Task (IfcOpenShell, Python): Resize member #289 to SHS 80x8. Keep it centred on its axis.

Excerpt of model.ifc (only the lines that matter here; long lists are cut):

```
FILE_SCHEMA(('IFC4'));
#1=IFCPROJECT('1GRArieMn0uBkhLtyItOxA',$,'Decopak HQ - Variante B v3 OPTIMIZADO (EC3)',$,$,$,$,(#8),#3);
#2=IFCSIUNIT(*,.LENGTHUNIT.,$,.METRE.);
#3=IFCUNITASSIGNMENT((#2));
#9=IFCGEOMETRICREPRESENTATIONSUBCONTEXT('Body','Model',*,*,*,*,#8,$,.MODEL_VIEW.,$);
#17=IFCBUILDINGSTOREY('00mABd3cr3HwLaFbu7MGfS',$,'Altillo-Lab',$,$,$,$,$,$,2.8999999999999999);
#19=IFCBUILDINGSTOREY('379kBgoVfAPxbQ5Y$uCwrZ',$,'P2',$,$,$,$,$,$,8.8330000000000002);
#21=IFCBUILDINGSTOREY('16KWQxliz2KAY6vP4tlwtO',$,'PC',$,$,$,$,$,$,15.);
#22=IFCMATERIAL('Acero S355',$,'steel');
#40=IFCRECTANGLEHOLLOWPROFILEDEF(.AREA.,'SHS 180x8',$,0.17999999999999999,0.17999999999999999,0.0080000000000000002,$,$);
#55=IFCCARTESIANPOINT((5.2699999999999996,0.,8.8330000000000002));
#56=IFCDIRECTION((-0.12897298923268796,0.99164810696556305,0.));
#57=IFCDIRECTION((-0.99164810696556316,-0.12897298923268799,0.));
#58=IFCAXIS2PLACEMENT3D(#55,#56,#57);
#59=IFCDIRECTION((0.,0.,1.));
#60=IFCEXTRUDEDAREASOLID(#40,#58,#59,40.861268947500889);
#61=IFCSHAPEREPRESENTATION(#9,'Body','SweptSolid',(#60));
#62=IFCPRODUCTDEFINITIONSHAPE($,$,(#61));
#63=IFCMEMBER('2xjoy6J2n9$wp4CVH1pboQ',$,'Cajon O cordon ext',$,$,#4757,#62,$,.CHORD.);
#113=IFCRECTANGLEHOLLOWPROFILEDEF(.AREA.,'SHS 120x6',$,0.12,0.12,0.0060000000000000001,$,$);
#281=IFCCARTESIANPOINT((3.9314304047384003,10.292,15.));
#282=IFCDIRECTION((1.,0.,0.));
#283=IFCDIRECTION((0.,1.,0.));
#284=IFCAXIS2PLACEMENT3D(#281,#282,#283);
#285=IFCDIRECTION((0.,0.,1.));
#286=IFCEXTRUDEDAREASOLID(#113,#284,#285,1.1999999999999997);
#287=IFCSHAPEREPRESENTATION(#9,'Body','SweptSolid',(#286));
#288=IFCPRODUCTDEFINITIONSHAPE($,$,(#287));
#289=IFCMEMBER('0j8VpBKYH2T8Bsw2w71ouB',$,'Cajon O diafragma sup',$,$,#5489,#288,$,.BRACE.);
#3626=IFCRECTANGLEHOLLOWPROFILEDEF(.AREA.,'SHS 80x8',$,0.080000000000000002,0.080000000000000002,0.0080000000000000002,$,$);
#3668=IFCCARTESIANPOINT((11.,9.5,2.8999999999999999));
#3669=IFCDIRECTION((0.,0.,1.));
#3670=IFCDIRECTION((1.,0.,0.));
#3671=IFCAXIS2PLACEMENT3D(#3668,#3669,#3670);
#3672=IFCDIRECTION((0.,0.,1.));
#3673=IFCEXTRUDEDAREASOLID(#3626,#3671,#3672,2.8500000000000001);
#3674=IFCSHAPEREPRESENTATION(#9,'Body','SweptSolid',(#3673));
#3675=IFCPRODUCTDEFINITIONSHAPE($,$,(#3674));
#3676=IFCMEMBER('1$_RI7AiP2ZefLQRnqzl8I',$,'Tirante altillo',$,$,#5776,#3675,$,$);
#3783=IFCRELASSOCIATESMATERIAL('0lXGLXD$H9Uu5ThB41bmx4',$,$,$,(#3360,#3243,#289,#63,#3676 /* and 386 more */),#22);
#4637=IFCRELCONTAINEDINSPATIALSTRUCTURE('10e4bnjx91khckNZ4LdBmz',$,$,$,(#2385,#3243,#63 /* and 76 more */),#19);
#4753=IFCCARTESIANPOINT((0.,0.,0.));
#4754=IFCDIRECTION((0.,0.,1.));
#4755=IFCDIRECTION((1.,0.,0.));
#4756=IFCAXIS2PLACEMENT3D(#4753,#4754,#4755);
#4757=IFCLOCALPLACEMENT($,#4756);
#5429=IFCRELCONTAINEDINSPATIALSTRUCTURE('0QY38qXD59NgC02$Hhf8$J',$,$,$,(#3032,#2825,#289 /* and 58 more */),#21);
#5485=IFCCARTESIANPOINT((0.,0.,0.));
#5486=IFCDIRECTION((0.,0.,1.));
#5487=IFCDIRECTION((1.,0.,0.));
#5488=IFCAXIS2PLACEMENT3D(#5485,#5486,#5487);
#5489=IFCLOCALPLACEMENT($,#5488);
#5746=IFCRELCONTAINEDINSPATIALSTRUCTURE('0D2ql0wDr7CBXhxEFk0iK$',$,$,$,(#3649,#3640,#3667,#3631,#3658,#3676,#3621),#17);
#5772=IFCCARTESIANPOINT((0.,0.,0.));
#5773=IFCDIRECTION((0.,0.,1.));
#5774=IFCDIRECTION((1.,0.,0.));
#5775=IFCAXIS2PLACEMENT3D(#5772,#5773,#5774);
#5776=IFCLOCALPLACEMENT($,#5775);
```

```python
import ifcopenshell
import ifcopenshell.util.element
import ifcopenshell.util.representation

model = ifcopenshell.open("model.ifc")

member = model.by_id(289)
source = next(p for p in model.by_type("IfcRectangleHollowProfileDef") if p.ProfileName == "SHS 80x8")

body = ifcopenshell.util.representation.get_representation(member, "Model", "Body")
solid = body.Items[0]
old_profile = solid.SweptArea

# Copy the section's sizes but keep this member's own profile position.
profile = ifcopenshell.util.element.copy(model, source)
profile.Position = old_profile.Position
solid.SweptArea = profile
if not model.get_total_inverses(old_profile):
    ifcopenshell.util.element.remove_deep2(model, old_profile)

print(solid.SweptArea)

model.write("model_v2.ifc")
```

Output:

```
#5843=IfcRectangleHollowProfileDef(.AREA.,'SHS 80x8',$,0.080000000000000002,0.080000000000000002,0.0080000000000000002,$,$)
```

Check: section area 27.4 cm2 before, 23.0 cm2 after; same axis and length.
